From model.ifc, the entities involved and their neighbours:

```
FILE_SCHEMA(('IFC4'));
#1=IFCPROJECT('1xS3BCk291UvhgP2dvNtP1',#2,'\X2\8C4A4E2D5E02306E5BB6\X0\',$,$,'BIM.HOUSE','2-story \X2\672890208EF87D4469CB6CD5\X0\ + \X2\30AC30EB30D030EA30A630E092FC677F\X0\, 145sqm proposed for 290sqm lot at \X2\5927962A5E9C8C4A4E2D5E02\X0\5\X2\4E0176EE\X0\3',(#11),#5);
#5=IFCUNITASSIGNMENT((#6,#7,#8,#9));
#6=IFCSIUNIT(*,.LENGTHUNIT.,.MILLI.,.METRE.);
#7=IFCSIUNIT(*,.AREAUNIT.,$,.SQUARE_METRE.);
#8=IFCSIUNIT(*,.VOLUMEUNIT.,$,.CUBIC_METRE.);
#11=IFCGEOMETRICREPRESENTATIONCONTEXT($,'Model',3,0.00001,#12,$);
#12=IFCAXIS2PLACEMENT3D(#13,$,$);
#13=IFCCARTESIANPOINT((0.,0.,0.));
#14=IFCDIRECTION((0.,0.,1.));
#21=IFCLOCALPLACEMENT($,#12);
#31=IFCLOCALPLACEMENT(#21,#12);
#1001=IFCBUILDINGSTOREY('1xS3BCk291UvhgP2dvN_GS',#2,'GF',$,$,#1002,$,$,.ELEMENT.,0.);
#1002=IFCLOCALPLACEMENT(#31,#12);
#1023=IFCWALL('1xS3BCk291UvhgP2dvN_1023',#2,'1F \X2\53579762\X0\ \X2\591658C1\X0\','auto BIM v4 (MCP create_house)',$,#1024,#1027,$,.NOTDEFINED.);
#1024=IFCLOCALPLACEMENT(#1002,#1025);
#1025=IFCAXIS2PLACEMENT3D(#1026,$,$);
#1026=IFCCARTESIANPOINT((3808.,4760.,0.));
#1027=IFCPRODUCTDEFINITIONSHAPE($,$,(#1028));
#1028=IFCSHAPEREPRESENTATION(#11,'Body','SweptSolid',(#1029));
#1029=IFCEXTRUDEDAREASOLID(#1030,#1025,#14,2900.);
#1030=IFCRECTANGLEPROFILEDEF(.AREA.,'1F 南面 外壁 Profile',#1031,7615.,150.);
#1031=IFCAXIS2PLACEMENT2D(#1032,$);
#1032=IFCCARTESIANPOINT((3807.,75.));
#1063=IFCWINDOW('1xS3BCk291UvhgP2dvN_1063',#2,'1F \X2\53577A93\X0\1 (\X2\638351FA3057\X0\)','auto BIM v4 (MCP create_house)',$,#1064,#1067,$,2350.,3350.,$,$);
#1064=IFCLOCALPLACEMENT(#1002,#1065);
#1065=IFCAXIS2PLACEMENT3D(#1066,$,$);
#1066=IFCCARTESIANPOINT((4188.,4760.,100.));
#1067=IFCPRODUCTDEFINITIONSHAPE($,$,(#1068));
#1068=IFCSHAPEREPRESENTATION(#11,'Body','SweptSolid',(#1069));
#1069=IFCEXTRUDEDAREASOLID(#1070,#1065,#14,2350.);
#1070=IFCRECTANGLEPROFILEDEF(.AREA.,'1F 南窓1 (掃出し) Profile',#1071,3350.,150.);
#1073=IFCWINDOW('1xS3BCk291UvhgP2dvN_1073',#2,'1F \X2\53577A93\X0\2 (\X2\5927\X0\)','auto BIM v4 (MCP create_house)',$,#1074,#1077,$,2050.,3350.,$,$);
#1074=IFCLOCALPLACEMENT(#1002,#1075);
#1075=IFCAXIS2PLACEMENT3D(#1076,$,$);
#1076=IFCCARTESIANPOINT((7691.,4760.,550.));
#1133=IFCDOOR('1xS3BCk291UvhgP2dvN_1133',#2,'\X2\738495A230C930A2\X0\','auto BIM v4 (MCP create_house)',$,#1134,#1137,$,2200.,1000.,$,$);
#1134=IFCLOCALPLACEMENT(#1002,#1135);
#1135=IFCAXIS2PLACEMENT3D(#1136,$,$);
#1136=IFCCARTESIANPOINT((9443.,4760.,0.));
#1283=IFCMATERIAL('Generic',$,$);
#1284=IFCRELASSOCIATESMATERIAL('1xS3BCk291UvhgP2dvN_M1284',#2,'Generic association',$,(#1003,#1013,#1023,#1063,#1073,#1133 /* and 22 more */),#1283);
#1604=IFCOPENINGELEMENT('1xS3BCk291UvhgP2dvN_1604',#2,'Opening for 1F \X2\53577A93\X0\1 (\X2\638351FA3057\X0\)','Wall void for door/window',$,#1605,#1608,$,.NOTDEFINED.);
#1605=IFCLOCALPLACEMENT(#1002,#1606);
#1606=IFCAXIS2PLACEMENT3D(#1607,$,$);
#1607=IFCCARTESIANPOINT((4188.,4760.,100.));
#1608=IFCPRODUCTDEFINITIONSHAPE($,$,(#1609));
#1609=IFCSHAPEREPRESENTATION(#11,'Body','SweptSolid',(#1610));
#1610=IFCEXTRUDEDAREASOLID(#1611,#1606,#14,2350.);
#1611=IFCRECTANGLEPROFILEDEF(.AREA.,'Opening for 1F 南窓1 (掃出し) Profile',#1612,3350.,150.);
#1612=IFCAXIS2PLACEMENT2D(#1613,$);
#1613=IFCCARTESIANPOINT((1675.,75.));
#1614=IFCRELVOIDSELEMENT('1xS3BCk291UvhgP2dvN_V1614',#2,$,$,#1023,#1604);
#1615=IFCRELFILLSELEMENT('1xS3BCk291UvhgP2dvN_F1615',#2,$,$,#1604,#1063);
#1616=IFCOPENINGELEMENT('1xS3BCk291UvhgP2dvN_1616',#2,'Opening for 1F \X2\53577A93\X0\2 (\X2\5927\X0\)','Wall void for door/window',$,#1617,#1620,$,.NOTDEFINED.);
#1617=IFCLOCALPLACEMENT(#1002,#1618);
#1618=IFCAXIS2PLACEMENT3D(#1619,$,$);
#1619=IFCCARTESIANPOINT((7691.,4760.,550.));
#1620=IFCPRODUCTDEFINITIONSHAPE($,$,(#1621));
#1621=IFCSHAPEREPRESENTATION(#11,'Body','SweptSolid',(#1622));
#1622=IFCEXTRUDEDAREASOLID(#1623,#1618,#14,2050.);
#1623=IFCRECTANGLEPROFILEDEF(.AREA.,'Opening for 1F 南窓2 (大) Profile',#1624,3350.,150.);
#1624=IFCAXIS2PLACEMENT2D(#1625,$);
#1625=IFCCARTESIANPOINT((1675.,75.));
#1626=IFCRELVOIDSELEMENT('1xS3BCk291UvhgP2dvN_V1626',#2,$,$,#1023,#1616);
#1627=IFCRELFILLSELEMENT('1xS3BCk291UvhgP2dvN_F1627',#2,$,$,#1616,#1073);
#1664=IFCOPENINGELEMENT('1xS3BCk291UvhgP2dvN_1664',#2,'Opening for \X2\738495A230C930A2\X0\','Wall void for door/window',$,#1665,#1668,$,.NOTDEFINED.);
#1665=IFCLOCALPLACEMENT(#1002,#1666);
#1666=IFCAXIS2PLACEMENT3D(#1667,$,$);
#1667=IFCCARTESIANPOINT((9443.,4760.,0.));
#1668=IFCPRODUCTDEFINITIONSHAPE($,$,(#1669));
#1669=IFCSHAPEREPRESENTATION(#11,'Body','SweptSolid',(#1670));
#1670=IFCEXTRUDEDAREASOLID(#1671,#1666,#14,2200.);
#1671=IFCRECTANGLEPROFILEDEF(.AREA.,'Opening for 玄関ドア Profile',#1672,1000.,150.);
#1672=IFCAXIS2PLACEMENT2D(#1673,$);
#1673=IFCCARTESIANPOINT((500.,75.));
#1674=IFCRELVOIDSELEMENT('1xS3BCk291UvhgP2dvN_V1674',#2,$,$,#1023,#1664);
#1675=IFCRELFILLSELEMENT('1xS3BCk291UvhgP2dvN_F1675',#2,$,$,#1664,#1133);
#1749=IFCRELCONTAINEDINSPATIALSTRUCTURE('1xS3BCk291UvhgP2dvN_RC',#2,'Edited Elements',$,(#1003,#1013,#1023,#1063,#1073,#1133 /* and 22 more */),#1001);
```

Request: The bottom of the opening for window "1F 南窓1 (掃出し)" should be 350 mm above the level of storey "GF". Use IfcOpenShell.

```python
import numpy as np
import ifcopenshell
import ifcopenshell.api.geometry
import ifcopenshell.geom
import ifcopenshell.util.element
import ifcopenshell.util.placement
import ifcopenshell.util.shape
import ifcopenshell.util.unit

model = ifcopenshell.open("model.ifc")
unit_scale = ifcopenshell.util.unit.calculate_unit_scale(model)

window = model.by_guid("1xS3BCk291UvhgP2dvN_1063")
opening = window.FillsVoids[0].RelatingOpeningElement
storey = ifcopenshell.util.element.get_container(window, ifc_class="IfcBuildingStorey")
level = ifcopenshell.util.placement.get_local_placement(storey.ObjectPlacement)[2, 3]

# The opening's origin need not be at the sill, so measure its lowest point.
shape = ifcopenshell.geom.create_shape(ifcopenshell.geom.settings(), opening)
bottom = ifcopenshell.util.shape.get_shape_bottom_elevation(shape, shape.geometry) / unit_scale
dz = level + 0.35 / unit_scale - bottom

shift = np.array([0.0, 0.0, dz])
# The window is not placed relative to its opening, so move both.
for product in (opening, window):
    matrix = ifcopenshell.util.placement.get_local_placement(product.ObjectPlacement)
    matrix[:3, 3] += shift
    ifcopenshell.api.geometry.edit_object_placement(model, product=product, matrix=matrix, is_si=False)

print(f"moved by {dz * unit_scale:+.3f} m")

model.write("model-out.ifc")
```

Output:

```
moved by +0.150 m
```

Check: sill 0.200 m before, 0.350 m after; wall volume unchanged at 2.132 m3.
